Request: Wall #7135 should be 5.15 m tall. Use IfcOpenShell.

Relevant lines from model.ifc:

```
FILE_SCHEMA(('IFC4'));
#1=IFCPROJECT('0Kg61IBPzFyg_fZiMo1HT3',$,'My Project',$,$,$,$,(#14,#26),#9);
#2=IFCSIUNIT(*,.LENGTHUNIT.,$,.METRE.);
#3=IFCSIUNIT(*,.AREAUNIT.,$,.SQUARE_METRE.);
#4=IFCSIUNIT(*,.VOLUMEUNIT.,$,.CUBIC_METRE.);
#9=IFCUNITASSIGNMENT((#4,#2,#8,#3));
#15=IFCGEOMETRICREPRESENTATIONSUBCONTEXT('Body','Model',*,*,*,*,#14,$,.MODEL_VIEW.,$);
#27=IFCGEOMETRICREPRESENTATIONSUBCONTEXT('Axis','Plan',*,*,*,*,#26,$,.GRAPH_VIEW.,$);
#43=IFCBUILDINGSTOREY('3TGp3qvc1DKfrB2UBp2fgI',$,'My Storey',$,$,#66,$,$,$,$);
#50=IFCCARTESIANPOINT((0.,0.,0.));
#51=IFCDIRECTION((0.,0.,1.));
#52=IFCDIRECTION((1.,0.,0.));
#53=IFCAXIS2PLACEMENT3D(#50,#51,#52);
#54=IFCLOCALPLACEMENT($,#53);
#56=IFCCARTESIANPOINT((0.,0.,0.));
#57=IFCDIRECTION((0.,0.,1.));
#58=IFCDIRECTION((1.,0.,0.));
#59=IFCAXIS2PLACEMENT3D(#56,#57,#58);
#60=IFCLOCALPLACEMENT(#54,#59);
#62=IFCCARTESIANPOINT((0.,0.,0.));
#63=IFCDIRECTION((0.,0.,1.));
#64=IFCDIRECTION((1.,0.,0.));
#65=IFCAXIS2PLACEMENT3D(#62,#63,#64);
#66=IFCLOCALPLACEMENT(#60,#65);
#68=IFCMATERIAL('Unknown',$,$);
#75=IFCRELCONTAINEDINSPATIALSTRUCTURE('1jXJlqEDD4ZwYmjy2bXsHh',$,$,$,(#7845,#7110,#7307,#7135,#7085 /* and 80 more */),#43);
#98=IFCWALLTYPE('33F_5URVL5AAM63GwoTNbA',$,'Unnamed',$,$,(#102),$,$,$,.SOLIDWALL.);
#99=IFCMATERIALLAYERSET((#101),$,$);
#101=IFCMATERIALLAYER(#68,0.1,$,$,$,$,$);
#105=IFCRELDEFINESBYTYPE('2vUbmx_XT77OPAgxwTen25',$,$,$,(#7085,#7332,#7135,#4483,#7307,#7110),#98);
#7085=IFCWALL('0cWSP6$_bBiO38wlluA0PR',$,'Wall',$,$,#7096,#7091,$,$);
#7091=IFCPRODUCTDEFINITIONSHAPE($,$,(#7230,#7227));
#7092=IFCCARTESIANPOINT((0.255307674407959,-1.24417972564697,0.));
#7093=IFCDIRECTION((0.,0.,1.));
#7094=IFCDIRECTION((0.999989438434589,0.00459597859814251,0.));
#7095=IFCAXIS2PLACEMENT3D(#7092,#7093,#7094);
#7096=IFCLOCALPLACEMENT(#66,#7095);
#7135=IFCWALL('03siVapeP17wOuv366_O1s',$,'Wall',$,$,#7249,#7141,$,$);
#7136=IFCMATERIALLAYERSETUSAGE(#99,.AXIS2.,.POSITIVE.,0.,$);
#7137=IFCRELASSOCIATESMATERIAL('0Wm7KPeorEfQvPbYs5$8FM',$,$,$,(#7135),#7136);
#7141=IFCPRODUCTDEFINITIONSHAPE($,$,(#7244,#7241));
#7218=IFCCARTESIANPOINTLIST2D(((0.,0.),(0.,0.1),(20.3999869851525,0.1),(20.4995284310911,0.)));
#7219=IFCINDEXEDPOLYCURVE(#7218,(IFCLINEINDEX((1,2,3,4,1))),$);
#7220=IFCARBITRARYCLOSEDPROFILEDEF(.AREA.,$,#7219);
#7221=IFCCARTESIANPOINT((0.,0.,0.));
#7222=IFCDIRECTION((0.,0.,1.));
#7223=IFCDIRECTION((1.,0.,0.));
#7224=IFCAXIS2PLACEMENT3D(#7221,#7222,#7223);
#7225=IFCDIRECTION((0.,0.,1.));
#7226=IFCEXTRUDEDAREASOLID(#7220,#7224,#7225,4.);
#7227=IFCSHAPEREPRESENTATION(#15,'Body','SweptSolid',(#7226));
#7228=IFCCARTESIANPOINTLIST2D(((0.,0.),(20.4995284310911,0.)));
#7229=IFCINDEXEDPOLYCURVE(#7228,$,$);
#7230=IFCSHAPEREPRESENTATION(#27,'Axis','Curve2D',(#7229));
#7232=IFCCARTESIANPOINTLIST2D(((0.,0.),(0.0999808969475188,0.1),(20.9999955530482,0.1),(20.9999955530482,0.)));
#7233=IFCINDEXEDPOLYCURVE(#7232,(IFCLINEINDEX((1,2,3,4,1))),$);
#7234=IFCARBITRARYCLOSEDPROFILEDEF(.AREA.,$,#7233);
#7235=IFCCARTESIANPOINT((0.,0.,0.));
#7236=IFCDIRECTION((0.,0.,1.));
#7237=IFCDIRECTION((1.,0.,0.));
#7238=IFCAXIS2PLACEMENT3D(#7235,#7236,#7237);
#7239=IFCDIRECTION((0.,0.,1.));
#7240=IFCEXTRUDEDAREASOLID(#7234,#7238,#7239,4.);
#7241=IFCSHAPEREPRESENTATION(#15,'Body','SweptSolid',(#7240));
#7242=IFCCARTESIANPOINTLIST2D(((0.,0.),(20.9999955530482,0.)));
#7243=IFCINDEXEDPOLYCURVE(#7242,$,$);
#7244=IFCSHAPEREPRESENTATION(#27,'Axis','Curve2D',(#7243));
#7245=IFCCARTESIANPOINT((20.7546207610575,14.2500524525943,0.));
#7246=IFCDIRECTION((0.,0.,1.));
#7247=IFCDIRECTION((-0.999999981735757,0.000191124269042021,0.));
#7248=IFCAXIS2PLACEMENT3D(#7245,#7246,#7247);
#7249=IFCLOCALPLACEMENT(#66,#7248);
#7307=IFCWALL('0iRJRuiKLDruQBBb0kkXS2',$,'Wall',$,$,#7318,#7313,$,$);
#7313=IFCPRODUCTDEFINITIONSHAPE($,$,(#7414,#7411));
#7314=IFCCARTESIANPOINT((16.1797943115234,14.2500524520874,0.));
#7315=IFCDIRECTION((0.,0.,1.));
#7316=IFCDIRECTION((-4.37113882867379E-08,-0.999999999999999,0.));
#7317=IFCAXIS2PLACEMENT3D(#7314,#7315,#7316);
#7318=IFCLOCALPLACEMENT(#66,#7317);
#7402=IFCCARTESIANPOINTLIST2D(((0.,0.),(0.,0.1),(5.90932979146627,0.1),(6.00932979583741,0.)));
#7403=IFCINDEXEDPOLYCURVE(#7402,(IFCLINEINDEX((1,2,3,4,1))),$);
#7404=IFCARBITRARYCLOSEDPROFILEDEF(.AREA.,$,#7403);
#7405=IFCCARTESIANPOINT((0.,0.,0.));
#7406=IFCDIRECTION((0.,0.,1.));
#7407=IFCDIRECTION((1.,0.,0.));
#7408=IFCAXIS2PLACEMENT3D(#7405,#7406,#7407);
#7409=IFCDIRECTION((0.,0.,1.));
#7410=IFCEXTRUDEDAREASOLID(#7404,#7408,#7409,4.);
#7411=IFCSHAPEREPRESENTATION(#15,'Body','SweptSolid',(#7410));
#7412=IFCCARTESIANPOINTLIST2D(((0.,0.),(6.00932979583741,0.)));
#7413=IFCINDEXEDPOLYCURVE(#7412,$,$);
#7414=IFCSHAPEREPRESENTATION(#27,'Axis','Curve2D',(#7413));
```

```python
import ifcopenshell
import ifcopenshell.geom
import ifcopenshell.util.representation
import ifcopenshell.util.shape
import ifcopenshell.util.unit

model = ifcopenshell.open("model.ifc")
unit_scale = ifcopenshell.util.unit.calculate_unit_scale(model)
settings = ifcopenshell.geom.settings()


def volume(element):
    """Net volume in cubic metres, openings subtracted."""
    shape = ifcopenshell.geom.create_shape(settings, element)
    return ifcopenshell.util.shape.get_volume(shape.geometry)


wall = model.by_id(7135)
before = volume(wall)

body = ifcopenshell.util.representation.get_representation(wall, "Model", "Body")
solid = body.Items[0]
old_height = solid.Depth
solid.Depth = 5.15 / unit_scale
after = volume(wall)

print(f"height {old_height:g} -> {solid.Depth:g}, volume {before:.3f} -> {after:.3f} m3")

model.write("model_rev.ifc")
```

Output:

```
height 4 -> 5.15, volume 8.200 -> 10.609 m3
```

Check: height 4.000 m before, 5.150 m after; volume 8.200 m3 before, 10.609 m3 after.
